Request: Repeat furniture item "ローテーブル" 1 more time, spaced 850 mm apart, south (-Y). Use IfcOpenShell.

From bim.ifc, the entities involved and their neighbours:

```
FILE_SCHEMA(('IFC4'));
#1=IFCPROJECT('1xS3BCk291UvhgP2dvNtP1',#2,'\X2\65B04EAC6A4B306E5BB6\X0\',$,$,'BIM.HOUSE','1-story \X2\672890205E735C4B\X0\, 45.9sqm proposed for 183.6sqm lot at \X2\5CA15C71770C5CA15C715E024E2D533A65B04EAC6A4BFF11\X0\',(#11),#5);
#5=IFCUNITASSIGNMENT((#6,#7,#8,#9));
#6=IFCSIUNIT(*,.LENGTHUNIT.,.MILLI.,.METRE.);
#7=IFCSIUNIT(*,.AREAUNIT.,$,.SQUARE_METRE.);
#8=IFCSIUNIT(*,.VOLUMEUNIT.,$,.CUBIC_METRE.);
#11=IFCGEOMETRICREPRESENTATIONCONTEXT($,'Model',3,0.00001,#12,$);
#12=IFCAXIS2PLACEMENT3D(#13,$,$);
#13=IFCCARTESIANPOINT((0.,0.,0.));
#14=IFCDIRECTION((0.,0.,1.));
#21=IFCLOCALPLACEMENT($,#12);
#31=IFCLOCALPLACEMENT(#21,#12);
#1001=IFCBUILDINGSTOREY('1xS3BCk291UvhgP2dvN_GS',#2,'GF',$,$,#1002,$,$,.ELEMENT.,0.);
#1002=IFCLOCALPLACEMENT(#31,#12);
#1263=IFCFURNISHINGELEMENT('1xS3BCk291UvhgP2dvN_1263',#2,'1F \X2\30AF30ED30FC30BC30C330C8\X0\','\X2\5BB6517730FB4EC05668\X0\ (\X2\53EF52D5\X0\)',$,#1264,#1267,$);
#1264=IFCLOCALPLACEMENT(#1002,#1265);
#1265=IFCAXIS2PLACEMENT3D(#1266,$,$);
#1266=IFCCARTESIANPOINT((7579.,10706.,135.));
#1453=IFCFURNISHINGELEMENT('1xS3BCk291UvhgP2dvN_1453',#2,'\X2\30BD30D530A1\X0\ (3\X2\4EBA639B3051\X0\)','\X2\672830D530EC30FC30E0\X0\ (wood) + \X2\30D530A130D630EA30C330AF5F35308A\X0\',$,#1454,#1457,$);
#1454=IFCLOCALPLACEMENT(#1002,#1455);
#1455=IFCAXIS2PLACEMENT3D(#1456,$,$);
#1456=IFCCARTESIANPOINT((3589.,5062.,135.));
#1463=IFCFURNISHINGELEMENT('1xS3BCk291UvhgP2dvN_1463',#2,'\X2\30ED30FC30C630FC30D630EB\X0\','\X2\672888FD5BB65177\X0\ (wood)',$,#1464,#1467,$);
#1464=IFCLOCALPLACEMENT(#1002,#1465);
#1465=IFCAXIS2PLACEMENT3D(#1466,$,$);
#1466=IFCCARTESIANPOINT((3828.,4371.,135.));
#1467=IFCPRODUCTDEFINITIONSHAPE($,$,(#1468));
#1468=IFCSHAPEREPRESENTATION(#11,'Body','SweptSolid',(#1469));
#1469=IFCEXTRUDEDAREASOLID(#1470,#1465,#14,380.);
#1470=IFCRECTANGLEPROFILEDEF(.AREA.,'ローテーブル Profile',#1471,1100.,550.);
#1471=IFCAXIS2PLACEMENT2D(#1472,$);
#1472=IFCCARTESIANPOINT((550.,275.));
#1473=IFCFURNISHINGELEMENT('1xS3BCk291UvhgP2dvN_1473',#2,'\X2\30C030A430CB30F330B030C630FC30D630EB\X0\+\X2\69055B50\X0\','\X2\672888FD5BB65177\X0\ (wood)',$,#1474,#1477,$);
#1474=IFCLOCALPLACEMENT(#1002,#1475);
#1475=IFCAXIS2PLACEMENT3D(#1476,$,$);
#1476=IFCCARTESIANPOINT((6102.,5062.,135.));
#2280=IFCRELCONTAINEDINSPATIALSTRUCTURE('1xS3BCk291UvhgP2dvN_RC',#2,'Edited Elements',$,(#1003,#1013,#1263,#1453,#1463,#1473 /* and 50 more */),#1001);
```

```python
import numpy as np
import ifcopenshell
import ifcopenshell.api.geometry
import ifcopenshell.api.root
import ifcopenshell.util.element
import ifcopenshell.util.placement
import ifcopenshell.util.unit

model = ifcopenshell.open("bim.ifc")
unit_scale = ifcopenshell.util.unit.calculate_unit_scale(model)


def reuse_history(source, copy):
    """copy_class also copies each property set's owner history, people and application; keep the originals."""
    for rel in copy.IsDefinedBy:
        if rel.is_a("IfcRelDefinesByProperties") and (history := rel.RelatingPropertyDefinition.OwnerHistory):
            rel.RelatingPropertyDefinition.OwnerHistory = source.OwnerHistory
            ifcopenshell.util.element.remove_deep2(model, history)


source = model.by_guid("1xS3BCk291UvhgP2dvN_1463")
base = ifcopenshell.util.placement.get_local_placement(source.ObjectPlacement)
step = np.array([0.0, -1.0, 0.0]) * 0.85 / unit_scale

for i in range(1, 2):
    copy = ifcopenshell.api.root.copy_class(model, product=source)
    copy.Representation = ifcopenshell.util.element.copy_deep(
        model, source.Representation, exclude=["IfcGeometricRepresentationContext", "IfcRepresentationMap"]
    )
    reuse_history(source, copy)
    matrix = base.copy()
    matrix[:3, 3] += i * step
    print("added at", matrix[:3, 3].round(3) + 0.0)
    ifcopenshell.api.geometry.edit_object_placement(model, product=copy, matrix=matrix, is_si=False)

model.write("bim-out.ifc")
```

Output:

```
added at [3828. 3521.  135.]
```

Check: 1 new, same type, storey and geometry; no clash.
